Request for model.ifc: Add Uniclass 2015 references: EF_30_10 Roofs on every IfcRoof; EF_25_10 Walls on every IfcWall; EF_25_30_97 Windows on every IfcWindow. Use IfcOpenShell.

First a look at what the model holds.

```python
import ifcopenshell

model = ifcopenshell.open("model.ifc")
print(model.schema)
print("classifications:", [c.Name for c in model.by_type("IfcClassification")])
for ifc_class in ("IfcDoor", "IfcRoof", "IfcStair", "IfcWall", "IfcWindow"):
    print(ifc_class, len(model.by_type(ifc_class)))
```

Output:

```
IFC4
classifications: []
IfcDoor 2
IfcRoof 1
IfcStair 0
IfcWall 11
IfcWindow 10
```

```python
import ifcopenshell
import ifcopenshell.api.classification

model = ifcopenshell.open("model.ifc")

system = ifcopenshell.api.classification.add_classification(model, classification="Uniclass 2015")

codes = {
    "IfcRoof": ("EF_30_10", "Roofs"),
    "IfcWall": ("EF_25_10", "Walls"),
    "IfcWindow": ("EF_25_30_97", "Windows"),
}
for ifc_class, (code, name) in codes.items():
    products = model.by_type(ifc_class)
    ifcopenshell.api.classification.add_reference(
        model, products=products, classification=system, identification=code, name=name
    )
    print(code, len(products))

model.write("model_v2.ifc")
```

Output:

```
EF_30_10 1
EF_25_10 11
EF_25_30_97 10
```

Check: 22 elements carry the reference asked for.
